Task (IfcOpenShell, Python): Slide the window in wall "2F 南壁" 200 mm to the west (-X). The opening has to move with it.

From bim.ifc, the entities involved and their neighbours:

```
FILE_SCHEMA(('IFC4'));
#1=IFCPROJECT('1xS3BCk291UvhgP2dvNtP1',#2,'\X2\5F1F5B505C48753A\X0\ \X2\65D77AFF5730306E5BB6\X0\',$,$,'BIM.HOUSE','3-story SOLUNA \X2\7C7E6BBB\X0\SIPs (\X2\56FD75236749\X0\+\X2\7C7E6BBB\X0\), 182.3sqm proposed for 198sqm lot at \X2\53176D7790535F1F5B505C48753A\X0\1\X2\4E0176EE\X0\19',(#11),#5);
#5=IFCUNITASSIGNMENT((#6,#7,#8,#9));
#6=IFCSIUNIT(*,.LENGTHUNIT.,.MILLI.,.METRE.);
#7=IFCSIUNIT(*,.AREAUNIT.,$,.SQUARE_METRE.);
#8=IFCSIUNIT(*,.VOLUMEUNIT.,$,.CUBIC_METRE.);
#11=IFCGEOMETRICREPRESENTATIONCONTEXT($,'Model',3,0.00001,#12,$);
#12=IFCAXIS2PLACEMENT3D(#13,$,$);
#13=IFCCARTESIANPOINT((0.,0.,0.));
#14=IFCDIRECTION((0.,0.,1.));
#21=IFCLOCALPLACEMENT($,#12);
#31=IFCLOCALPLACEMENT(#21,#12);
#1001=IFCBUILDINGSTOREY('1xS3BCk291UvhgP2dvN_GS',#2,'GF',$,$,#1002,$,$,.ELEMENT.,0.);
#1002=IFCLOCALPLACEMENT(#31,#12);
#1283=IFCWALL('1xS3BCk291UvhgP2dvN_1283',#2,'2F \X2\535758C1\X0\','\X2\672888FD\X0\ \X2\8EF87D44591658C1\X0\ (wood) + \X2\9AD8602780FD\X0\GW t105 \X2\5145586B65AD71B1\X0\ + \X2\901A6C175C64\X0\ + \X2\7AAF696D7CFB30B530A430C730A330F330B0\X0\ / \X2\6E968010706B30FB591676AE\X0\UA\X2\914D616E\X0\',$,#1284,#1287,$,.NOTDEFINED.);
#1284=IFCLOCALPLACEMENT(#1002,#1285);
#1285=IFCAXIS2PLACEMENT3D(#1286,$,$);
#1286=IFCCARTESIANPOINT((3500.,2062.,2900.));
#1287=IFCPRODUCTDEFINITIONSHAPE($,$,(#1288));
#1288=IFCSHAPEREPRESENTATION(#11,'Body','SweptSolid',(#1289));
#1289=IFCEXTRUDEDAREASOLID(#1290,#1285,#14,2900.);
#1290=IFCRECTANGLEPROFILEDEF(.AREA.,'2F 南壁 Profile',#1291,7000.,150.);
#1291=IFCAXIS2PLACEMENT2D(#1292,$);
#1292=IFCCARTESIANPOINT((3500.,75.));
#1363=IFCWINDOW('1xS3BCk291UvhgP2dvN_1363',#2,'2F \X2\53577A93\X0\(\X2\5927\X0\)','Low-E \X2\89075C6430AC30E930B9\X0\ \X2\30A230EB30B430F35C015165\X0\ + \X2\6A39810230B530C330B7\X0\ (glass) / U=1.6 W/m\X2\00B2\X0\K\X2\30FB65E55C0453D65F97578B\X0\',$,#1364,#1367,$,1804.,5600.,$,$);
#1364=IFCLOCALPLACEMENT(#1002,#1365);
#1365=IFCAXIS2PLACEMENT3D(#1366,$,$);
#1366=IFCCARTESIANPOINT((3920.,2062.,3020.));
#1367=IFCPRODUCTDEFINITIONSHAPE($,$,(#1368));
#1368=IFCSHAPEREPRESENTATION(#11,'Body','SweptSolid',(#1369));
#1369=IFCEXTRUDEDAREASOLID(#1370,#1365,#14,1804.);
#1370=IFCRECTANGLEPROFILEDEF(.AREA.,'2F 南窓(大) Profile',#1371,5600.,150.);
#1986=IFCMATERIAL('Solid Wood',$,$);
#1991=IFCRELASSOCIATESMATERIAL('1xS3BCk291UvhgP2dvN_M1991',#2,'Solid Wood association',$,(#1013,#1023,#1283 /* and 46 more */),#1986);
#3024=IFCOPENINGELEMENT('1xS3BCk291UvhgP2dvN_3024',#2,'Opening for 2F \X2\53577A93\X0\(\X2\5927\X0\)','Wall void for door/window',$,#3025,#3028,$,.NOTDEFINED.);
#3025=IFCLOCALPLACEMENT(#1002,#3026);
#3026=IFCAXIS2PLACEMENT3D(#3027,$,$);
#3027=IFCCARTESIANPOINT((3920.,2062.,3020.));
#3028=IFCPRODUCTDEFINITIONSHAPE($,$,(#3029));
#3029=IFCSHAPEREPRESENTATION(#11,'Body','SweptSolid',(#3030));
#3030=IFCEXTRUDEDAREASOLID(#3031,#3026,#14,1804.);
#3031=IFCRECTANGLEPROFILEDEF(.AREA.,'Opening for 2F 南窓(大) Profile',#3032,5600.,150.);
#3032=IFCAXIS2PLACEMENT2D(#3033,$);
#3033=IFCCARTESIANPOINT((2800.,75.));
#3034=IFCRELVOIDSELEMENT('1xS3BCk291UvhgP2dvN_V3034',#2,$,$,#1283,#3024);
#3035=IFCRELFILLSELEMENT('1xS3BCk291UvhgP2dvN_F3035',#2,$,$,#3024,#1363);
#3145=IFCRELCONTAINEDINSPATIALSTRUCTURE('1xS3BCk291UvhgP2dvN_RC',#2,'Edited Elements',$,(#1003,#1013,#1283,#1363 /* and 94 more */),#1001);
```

```python
import ifcopenshell
import ifcopenshell.api.geometry
import ifcopenshell.util.placement

model = ifcopenshell.open("bim.ifc")

window = model.by_guid("1xS3BCk291UvhgP2dvN_1363")
opening = window.FillsVoids[0].RelatingOpeningElement
wall = opening.VoidsElements[0].RelatingBuildingElement

wall_matrix = ifcopenshell.util.placement.get_local_placement(wall.ObjectPlacement)
shift = wall_matrix[:3, 0] * -200.0
before = ifcopenshell.util.placement.get_local_placement(window.ObjectPlacement)[:3, 3].copy()

# The window is not placed relative to its opening, so move both.
for product in (opening, window):
    matrix = ifcopenshell.util.placement.get_local_placement(product.ObjectPlacement)
    matrix[:3, 3] += shift
    ifcopenshell.api.geometry.edit_object_placement(model, product=product, matrix=matrix, is_si=False)

after = ifcopenshell.util.placement.get_local_placement(window.ObjectPlacement)[:3, 3]
print("window moved by", (after - before).round(3) + 0.0)

model.write("bim-out.ifc")
```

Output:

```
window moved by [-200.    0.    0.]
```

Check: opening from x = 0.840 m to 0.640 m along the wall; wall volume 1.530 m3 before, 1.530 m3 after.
